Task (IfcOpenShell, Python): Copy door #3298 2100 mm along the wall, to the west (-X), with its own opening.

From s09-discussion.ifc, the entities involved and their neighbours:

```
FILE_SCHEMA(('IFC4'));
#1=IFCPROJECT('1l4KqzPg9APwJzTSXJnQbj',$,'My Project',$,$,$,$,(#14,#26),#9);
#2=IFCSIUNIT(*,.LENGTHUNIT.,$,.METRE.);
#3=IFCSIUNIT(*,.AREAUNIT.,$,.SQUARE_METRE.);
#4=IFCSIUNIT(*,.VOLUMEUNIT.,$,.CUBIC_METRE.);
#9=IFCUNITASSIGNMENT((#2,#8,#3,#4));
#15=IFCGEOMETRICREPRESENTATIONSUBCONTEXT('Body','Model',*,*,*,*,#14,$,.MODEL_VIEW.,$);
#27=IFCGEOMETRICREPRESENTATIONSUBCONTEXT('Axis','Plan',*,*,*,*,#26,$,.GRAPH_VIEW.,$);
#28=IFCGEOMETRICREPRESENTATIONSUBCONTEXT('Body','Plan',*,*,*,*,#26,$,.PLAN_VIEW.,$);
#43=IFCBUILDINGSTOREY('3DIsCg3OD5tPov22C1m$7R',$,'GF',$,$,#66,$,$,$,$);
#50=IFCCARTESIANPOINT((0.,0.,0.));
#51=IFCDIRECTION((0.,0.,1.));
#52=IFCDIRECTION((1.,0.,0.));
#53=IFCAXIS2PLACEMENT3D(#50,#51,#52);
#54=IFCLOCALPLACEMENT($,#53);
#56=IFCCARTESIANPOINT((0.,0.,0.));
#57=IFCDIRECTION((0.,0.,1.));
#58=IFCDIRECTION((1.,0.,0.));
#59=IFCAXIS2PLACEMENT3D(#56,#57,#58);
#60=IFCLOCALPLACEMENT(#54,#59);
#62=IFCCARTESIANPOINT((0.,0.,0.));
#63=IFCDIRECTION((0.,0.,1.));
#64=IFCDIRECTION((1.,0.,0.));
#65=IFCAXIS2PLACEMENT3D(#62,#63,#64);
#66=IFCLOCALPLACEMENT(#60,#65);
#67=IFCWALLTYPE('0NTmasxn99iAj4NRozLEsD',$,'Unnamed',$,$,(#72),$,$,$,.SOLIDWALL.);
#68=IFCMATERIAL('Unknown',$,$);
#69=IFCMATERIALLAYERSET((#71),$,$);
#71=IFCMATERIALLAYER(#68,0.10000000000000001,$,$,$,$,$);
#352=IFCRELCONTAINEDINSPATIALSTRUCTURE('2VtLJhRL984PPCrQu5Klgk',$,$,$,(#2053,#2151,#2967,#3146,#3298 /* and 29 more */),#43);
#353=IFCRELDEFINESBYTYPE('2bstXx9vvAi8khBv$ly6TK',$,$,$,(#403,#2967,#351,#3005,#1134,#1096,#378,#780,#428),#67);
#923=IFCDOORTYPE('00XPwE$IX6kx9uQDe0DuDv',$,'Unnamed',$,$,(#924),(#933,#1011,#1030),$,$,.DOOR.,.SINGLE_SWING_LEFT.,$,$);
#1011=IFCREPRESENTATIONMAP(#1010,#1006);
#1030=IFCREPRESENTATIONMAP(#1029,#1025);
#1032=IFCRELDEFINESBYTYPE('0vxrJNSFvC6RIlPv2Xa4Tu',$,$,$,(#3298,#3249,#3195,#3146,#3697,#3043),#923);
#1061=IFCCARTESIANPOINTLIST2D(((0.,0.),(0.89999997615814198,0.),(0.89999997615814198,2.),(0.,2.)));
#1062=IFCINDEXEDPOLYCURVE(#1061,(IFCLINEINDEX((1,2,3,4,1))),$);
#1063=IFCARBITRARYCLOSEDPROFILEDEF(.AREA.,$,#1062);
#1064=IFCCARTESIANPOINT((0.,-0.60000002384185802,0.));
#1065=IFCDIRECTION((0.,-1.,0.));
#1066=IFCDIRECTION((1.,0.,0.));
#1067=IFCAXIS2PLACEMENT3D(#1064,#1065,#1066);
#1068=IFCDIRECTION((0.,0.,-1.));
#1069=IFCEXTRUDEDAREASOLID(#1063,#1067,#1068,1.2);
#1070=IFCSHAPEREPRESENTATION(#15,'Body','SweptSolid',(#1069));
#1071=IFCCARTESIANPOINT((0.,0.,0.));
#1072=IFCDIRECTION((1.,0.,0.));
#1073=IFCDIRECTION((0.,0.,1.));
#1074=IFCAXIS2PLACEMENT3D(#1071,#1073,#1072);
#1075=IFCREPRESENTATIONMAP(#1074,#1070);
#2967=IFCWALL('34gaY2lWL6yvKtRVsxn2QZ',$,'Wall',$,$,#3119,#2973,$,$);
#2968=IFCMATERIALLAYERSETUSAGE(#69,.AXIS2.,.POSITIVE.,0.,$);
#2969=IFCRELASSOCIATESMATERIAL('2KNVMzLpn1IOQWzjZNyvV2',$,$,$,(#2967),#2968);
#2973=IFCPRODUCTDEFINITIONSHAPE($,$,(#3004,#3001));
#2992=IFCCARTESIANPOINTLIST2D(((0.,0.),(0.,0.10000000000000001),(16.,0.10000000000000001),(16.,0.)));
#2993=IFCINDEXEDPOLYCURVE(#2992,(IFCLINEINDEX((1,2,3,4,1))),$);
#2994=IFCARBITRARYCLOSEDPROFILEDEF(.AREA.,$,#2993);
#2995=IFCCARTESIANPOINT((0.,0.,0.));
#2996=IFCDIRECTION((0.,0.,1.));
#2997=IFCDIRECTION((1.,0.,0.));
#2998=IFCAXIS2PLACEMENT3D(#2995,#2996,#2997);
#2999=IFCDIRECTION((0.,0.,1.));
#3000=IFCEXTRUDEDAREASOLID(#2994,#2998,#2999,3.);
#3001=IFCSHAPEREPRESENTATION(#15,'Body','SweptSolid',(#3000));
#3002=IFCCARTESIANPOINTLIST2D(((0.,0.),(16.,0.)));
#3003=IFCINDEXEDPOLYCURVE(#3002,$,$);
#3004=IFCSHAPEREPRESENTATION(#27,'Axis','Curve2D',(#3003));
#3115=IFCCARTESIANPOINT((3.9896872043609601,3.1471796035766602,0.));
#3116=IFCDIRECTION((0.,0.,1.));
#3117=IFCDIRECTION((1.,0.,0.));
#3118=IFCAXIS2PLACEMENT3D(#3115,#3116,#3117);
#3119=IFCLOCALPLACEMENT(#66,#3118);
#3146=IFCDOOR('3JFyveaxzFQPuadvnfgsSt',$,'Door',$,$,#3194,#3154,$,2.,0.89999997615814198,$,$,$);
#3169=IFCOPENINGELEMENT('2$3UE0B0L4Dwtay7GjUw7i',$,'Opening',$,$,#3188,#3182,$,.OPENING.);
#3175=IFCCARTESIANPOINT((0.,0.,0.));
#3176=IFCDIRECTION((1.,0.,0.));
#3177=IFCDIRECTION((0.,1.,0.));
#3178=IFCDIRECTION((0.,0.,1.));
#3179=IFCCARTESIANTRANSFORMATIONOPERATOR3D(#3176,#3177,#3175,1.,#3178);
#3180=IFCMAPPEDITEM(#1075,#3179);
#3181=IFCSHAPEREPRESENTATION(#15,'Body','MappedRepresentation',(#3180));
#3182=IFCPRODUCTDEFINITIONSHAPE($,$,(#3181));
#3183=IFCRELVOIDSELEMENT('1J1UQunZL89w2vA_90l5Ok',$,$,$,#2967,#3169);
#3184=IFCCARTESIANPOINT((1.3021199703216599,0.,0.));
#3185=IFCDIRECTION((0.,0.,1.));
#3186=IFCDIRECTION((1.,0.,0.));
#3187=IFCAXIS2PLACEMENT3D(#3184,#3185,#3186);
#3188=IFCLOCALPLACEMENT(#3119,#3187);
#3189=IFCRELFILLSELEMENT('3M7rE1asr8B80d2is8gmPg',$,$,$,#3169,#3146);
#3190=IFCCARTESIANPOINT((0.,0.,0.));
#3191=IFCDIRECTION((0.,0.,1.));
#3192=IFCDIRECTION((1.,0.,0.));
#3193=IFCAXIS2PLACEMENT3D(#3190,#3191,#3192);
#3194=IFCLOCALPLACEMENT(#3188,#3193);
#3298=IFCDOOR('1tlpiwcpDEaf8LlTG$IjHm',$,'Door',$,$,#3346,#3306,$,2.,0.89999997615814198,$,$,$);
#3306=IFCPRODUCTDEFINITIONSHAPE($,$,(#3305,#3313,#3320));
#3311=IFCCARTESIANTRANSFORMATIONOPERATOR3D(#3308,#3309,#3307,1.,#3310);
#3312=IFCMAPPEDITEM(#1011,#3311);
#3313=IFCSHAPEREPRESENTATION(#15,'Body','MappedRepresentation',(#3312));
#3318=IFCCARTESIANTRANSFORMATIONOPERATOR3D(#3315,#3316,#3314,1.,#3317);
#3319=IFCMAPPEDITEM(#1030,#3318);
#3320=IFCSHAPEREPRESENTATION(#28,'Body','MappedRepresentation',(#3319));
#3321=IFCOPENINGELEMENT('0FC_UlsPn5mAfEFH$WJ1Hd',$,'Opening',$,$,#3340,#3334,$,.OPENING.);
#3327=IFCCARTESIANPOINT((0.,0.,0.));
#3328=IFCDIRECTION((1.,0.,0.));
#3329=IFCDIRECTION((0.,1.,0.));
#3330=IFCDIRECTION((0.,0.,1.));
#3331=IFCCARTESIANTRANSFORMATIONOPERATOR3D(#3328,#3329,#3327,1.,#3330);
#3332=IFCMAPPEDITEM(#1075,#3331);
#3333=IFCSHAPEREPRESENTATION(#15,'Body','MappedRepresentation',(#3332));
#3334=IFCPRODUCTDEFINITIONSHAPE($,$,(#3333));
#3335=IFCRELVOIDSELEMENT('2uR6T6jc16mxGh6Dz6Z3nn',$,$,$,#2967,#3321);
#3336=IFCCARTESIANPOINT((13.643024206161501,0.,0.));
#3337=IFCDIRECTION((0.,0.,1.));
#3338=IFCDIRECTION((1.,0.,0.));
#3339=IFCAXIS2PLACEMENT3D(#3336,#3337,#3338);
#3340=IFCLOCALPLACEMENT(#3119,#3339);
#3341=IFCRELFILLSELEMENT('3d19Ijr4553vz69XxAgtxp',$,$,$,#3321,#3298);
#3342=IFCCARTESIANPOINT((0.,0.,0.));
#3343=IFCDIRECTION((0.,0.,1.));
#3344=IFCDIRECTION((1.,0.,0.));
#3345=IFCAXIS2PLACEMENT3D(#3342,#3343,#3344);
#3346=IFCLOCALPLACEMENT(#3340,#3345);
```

```python
import ifcopenshell
import ifcopenshell.api.feature
import ifcopenshell.api.geometry
import ifcopenshell.api.root
import ifcopenshell.geom
import ifcopenshell.util.element
import ifcopenshell.util.placement
import ifcopenshell.util.shape

model = ifcopenshell.open("s09-discussion.ifc")
settings = ifcopenshell.geom.settings()


def volume(element):
    """Net volume in cubic metres, openings subtracted."""
    shape = ifcopenshell.geom.create_shape(settings, element)
    return ifcopenshell.util.shape.get_volume(shape.geometry)


door = model.by_guid("1tlpiwcpDEaf8LlTG$IjHm")
opening = door.FillsVoids[0].RelatingOpeningElement
wall = opening.VoidsElements[0].RelatingBuildingElement
before = volume(wall)
shift = ifcopenshell.util.placement.get_local_placement(wall.ObjectPlacement)[:3, 0] * -2.1

# copy_class copies the void relationship, type, container and properties, but no geometry.
new_opening = ifcopenshell.api.root.copy_class(model, product=opening)
new_opening.Representation = ifcopenshell.util.element.copy_deep(
    model, opening.Representation, exclude=["IfcGeometricRepresentationContext", "IfcRepresentationMap"]
)
new_door = ifcopenshell.api.root.copy_class(model, product=door)
new_door.Representation = ifcopenshell.util.element.copy_deep(
    model, door.Representation, exclude=["IfcGeometricRepresentationContext", "IfcRepresentationMap"]
)
ifcopenshell.api.feature.add_filling(model, opening=new_opening, element=new_door)

for old, new in ((opening, new_opening), (door, new_door)):
    matrix = ifcopenshell.util.placement.get_local_placement(old.ObjectPlacement)
    matrix[:3, 3] += shift
    ifcopenshell.api.geometry.edit_object_placement(model, product=new, matrix=matrix, is_si=False)

after = volume(wall)

print(f"wall volume {before:.3f} -> {after:.3f} m3")

model.write("s09-discussion_v2.ifc")
```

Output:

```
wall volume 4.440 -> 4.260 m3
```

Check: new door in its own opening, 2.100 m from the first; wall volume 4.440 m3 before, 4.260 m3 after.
